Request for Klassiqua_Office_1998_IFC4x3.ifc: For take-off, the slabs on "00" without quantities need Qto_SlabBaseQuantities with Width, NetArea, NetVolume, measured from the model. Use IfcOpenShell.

First a look at what the model holds.

```python
import ifcopenshell
import ifcopenshell.util.element
import ifcopenshell.util.unit

model = ifcopenshell.open("Klassiqua_Office_1998_IFC4x3.ifc")
print(model.schema)
for unit_type in ("LENGTHUNIT", "AREAUNIT", "VOLUMEUNIT"):
    print(unit_type, ifcopenshell.util.unit.calculate_unit_scale(model, unit_type))
storey = next(s for s in model.by_type("IfcBuildingStorey") if s.Name == "00")
slabs = [e for e in ifcopenshell.util.element.get_decomposition(storey) if e.is_a("IfcSlab")]
for e in sorted(slabs, key=lambda e: e.id()):
    print(e.id(), e.is_a(), e.Name, list(ifcopenshell.util.element.get_psets(e, qtos_only=True)), sep=" | ")
```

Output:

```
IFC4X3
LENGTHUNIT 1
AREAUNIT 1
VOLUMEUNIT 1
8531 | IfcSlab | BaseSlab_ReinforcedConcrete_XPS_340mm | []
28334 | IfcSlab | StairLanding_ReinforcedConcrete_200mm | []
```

```python
import ifcopenshell
import ifcopenshell.api.pset
import ifcopenshell.geom
import ifcopenshell.util.element
import ifcopenshell.util.shape
import ifcopenshell.util.unit

model = ifcopenshell.open("Klassiqua_Office_1998_IFC4x3.ifc")
unit_scale = ifcopenshell.util.unit.calculate_unit_scale(model)
area_scale = ifcopenshell.util.unit.calculate_unit_scale(model, "AREAUNIT")
volume_scale = ifcopenshell.util.unit.calculate_unit_scale(model, "VOLUMEUNIT")
settings = ifcopenshell.geom.settings()

storey = next(s for s in model.by_type("IfcBuildingStorey") if s.Name == "00")
slabs = [e for e in ifcopenshell.util.element.get_decomposition(storey) if e.is_a("IfcSlab")]

for e in sorted(slabs, key=lambda e: e.id()):
    if ifcopenshell.util.element.get_psets(e, qtos_only=True, should_inherit=False):
        continue
    # Geometry comes back in metres, in the element's own axes.
    shape = ifcopenshell.geom.create_shape(settings, e)
    values = {
        "Width": ifcopenshell.util.shape.get_z(shape.geometry) / unit_scale,
        "NetArea": ifcopenshell.util.shape.get_footprint_area(shape.geometry) / area_scale,
        "NetVolume": ifcopenshell.util.shape.get_volume(shape.geometry) / volume_scale,
    }
    qto = ifcopenshell.api.pset.add_qto(model, product=e, name="Qto_SlabBaseQuantities")
    ifcopenshell.api.pset.edit_qto(model, qto=qto, properties=values)
    print(e.id(), {k: round(v, 3) for k, v in values.items()})

model.write("Klassiqua_Office_1998_IFC4x3_updated.ifc")
```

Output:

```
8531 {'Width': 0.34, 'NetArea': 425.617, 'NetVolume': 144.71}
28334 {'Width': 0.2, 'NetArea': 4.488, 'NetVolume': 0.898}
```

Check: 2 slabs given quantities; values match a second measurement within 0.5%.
